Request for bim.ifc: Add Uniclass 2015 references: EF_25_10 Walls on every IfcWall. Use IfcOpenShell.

First a look at what the model holds.

```python
import ifcopenshell

model = ifcopenshell.open("bim.ifc")
print(model.schema)
print("classifications:", [c.Name for c in model.by_type("IfcClassification")])
for ifc_class in ("IfcDoor", "IfcRoof", "IfcStair", "IfcWall", "IfcWindow"):
    print(ifc_class, len(model.by_type(ifc_class)))
```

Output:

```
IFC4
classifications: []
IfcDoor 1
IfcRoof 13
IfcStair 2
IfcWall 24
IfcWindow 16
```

```python
import ifcopenshell
import ifcopenshell.api.classification

model = ifcopenshell.open("bim.ifc")

system = ifcopenshell.api.classification.add_classification(model, classification="Uniclass 2015")

codes = {
    "IfcWall": ("EF_25_10", "Walls"),
}
for ifc_class, (code, name) in codes.items():
    products = model.by_type(ifc_class)
    ifcopenshell.api.classification.add_reference(
        model, products=products, classification=system, identification=code, name=name
    )
    print(code, len(products))

model.write("bim_v2.ifc")
```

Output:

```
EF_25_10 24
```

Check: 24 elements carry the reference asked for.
